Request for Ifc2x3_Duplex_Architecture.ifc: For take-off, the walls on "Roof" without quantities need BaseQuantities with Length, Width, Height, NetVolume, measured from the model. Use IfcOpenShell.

First a look at what the model holds.

```python
import ifcopenshell
import ifcopenshell.util.element
import ifcopenshell.util.unit

model = ifcopenshell.open("Ifc2x3_Duplex_Architecture.ifc")
print(model.schema)
for unit_type in ("LENGTHUNIT", "AREAUNIT", "VOLUMEUNIT"):
    print(unit_type, ifcopenshell.util.unit.calculate_unit_scale(model, unit_type))
storey = next(s for s in model.by_type("IfcBuildingStorey") if s.Name == "Roof")
walls = [e for e in ifcopenshell.util.element.get_decomposition(storey) if e.is_a("IfcWall")]
for e in sorted(walls, key=lambda e: e.id()):
    print(e.id(), e.is_a(), e.Name, list(ifcopenshell.util.element.get_psets(e, qtos_only=True)), sep=" | ")
```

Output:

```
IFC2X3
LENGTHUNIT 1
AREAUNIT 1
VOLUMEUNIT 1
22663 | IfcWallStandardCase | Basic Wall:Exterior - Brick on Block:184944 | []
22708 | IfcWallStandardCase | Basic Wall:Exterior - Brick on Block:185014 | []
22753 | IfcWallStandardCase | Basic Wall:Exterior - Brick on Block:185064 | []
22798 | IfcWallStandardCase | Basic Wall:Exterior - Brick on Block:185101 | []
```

```python
import ifcopenshell
import ifcopenshell.api.pset
import ifcopenshell.geom
import ifcopenshell.util.element
import ifcopenshell.util.shape
import ifcopenshell.util.unit

model = ifcopenshell.open("Ifc2x3_Duplex_Architecture.ifc")
unit_scale = ifcopenshell.util.unit.calculate_unit_scale(model)
volume_scale = ifcopenshell.util.unit.calculate_unit_scale(model, "VOLUMEUNIT")
settings = ifcopenshell.geom.settings()

storey = next(s for s in model.by_type("IfcBuildingStorey") if s.Name == "Roof")
walls = [e for e in ifcopenshell.util.element.get_decomposition(storey) if e.is_a("IfcWall")]

for e in sorted(walls, key=lambda e: e.id()):
    if ifcopenshell.util.element.get_psets(e, qtos_only=True, should_inherit=False):
        continue
    # Geometry comes back in metres, in the element's own axes.
    shape = ifcopenshell.geom.create_shape(settings, e)
    values = {
        "Length": ifcopenshell.util.shape.get_x(shape.geometry) / unit_scale,
        "Width": ifcopenshell.util.shape.get_y(shape.geometry) / unit_scale,
        "Height": ifcopenshell.util.shape.get_z(shape.geometry) / unit_scale,
        "NetVolume": ifcopenshell.util.shape.get_volume(shape.geometry) / volume_scale,
    }
    qto = ifcopenshell.api.pset.add_qto(model, product=e, name="BaseQuantities")
    ifcopenshell.api.pset.edit_qto(model, qto=qto, properties=values)
    print(e.id(), {k: round(v, 3) for k, v in values.items()})

model.write("Ifc2x3_Duplex_Architecture_updated.ifc")
```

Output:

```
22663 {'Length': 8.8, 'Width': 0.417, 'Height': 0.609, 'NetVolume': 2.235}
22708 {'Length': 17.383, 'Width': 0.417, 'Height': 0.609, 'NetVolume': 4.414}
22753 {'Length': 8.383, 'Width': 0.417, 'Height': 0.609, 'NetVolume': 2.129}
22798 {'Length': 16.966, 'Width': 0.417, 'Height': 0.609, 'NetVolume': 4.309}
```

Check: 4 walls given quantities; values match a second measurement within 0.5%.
